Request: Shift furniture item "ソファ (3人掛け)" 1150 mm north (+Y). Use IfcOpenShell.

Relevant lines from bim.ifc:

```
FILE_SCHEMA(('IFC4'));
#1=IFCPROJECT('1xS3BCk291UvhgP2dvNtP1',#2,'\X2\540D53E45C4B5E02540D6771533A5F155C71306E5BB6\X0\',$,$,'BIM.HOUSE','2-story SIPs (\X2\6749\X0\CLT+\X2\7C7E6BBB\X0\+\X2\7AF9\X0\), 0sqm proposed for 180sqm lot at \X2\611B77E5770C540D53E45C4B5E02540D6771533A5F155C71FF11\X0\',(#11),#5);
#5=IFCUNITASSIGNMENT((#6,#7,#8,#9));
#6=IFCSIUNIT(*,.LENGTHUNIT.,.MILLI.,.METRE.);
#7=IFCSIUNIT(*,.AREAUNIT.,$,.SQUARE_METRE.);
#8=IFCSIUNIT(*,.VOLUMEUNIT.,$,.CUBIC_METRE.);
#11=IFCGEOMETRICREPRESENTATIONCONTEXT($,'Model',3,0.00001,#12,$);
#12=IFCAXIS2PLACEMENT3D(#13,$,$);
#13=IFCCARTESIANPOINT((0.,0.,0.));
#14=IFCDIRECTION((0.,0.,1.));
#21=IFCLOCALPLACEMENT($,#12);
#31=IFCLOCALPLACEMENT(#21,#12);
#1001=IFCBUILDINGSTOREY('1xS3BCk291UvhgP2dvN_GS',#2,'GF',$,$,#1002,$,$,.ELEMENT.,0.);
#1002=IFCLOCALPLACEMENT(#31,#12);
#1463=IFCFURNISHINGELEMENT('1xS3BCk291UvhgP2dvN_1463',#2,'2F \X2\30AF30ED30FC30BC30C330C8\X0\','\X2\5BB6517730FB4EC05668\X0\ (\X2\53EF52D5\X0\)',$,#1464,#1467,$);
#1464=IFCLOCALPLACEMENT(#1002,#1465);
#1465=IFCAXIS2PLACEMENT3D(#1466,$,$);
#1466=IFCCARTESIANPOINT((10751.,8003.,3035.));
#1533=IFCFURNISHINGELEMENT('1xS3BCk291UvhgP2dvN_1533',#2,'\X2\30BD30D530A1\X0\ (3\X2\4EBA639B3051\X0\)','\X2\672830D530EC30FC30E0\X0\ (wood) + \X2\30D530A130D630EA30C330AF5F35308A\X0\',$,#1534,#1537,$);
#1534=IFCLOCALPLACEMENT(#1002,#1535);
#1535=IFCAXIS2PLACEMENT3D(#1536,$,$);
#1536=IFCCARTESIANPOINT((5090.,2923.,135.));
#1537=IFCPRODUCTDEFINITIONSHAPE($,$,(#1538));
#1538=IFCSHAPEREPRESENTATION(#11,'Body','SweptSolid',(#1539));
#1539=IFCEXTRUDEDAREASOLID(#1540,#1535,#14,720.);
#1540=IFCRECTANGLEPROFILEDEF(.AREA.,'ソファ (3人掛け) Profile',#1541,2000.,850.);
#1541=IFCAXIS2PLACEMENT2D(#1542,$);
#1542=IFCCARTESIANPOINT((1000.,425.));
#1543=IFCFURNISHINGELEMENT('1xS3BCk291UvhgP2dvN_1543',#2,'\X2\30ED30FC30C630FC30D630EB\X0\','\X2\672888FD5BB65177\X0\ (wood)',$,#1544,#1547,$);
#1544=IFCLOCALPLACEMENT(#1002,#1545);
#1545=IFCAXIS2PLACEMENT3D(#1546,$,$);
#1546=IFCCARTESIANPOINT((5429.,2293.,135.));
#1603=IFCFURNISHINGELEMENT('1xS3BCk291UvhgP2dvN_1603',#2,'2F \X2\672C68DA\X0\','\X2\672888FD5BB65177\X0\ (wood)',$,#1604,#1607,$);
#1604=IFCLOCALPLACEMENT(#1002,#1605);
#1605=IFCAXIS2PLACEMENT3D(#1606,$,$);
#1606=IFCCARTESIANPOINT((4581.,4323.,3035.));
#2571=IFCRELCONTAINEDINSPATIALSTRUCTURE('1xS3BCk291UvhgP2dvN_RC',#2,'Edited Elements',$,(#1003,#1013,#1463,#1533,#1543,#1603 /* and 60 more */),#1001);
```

```python
import ifcopenshell
import ifcopenshell.api.geometry
import ifcopenshell.util.placement

model = ifcopenshell.open("bim.ifc")

item = model.by_guid("1xS3BCk291UvhgP2dvN_1533")
matrix = ifcopenshell.util.placement.get_local_placement(item.ObjectPlacement)
matrix[1, 3] += 1150.0
ifcopenshell.api.geometry.edit_object_placement(model, product=item, matrix=matrix, is_si=False)

print(ifcopenshell.util.placement.get_local_placement(item.ObjectPlacement).round(3) + 0.0)

model.write("bim_rev.ifc")
```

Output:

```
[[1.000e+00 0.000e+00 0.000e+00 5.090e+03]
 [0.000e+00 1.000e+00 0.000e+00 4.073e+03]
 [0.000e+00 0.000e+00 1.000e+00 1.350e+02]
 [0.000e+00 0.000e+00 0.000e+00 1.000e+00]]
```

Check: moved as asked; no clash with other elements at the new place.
